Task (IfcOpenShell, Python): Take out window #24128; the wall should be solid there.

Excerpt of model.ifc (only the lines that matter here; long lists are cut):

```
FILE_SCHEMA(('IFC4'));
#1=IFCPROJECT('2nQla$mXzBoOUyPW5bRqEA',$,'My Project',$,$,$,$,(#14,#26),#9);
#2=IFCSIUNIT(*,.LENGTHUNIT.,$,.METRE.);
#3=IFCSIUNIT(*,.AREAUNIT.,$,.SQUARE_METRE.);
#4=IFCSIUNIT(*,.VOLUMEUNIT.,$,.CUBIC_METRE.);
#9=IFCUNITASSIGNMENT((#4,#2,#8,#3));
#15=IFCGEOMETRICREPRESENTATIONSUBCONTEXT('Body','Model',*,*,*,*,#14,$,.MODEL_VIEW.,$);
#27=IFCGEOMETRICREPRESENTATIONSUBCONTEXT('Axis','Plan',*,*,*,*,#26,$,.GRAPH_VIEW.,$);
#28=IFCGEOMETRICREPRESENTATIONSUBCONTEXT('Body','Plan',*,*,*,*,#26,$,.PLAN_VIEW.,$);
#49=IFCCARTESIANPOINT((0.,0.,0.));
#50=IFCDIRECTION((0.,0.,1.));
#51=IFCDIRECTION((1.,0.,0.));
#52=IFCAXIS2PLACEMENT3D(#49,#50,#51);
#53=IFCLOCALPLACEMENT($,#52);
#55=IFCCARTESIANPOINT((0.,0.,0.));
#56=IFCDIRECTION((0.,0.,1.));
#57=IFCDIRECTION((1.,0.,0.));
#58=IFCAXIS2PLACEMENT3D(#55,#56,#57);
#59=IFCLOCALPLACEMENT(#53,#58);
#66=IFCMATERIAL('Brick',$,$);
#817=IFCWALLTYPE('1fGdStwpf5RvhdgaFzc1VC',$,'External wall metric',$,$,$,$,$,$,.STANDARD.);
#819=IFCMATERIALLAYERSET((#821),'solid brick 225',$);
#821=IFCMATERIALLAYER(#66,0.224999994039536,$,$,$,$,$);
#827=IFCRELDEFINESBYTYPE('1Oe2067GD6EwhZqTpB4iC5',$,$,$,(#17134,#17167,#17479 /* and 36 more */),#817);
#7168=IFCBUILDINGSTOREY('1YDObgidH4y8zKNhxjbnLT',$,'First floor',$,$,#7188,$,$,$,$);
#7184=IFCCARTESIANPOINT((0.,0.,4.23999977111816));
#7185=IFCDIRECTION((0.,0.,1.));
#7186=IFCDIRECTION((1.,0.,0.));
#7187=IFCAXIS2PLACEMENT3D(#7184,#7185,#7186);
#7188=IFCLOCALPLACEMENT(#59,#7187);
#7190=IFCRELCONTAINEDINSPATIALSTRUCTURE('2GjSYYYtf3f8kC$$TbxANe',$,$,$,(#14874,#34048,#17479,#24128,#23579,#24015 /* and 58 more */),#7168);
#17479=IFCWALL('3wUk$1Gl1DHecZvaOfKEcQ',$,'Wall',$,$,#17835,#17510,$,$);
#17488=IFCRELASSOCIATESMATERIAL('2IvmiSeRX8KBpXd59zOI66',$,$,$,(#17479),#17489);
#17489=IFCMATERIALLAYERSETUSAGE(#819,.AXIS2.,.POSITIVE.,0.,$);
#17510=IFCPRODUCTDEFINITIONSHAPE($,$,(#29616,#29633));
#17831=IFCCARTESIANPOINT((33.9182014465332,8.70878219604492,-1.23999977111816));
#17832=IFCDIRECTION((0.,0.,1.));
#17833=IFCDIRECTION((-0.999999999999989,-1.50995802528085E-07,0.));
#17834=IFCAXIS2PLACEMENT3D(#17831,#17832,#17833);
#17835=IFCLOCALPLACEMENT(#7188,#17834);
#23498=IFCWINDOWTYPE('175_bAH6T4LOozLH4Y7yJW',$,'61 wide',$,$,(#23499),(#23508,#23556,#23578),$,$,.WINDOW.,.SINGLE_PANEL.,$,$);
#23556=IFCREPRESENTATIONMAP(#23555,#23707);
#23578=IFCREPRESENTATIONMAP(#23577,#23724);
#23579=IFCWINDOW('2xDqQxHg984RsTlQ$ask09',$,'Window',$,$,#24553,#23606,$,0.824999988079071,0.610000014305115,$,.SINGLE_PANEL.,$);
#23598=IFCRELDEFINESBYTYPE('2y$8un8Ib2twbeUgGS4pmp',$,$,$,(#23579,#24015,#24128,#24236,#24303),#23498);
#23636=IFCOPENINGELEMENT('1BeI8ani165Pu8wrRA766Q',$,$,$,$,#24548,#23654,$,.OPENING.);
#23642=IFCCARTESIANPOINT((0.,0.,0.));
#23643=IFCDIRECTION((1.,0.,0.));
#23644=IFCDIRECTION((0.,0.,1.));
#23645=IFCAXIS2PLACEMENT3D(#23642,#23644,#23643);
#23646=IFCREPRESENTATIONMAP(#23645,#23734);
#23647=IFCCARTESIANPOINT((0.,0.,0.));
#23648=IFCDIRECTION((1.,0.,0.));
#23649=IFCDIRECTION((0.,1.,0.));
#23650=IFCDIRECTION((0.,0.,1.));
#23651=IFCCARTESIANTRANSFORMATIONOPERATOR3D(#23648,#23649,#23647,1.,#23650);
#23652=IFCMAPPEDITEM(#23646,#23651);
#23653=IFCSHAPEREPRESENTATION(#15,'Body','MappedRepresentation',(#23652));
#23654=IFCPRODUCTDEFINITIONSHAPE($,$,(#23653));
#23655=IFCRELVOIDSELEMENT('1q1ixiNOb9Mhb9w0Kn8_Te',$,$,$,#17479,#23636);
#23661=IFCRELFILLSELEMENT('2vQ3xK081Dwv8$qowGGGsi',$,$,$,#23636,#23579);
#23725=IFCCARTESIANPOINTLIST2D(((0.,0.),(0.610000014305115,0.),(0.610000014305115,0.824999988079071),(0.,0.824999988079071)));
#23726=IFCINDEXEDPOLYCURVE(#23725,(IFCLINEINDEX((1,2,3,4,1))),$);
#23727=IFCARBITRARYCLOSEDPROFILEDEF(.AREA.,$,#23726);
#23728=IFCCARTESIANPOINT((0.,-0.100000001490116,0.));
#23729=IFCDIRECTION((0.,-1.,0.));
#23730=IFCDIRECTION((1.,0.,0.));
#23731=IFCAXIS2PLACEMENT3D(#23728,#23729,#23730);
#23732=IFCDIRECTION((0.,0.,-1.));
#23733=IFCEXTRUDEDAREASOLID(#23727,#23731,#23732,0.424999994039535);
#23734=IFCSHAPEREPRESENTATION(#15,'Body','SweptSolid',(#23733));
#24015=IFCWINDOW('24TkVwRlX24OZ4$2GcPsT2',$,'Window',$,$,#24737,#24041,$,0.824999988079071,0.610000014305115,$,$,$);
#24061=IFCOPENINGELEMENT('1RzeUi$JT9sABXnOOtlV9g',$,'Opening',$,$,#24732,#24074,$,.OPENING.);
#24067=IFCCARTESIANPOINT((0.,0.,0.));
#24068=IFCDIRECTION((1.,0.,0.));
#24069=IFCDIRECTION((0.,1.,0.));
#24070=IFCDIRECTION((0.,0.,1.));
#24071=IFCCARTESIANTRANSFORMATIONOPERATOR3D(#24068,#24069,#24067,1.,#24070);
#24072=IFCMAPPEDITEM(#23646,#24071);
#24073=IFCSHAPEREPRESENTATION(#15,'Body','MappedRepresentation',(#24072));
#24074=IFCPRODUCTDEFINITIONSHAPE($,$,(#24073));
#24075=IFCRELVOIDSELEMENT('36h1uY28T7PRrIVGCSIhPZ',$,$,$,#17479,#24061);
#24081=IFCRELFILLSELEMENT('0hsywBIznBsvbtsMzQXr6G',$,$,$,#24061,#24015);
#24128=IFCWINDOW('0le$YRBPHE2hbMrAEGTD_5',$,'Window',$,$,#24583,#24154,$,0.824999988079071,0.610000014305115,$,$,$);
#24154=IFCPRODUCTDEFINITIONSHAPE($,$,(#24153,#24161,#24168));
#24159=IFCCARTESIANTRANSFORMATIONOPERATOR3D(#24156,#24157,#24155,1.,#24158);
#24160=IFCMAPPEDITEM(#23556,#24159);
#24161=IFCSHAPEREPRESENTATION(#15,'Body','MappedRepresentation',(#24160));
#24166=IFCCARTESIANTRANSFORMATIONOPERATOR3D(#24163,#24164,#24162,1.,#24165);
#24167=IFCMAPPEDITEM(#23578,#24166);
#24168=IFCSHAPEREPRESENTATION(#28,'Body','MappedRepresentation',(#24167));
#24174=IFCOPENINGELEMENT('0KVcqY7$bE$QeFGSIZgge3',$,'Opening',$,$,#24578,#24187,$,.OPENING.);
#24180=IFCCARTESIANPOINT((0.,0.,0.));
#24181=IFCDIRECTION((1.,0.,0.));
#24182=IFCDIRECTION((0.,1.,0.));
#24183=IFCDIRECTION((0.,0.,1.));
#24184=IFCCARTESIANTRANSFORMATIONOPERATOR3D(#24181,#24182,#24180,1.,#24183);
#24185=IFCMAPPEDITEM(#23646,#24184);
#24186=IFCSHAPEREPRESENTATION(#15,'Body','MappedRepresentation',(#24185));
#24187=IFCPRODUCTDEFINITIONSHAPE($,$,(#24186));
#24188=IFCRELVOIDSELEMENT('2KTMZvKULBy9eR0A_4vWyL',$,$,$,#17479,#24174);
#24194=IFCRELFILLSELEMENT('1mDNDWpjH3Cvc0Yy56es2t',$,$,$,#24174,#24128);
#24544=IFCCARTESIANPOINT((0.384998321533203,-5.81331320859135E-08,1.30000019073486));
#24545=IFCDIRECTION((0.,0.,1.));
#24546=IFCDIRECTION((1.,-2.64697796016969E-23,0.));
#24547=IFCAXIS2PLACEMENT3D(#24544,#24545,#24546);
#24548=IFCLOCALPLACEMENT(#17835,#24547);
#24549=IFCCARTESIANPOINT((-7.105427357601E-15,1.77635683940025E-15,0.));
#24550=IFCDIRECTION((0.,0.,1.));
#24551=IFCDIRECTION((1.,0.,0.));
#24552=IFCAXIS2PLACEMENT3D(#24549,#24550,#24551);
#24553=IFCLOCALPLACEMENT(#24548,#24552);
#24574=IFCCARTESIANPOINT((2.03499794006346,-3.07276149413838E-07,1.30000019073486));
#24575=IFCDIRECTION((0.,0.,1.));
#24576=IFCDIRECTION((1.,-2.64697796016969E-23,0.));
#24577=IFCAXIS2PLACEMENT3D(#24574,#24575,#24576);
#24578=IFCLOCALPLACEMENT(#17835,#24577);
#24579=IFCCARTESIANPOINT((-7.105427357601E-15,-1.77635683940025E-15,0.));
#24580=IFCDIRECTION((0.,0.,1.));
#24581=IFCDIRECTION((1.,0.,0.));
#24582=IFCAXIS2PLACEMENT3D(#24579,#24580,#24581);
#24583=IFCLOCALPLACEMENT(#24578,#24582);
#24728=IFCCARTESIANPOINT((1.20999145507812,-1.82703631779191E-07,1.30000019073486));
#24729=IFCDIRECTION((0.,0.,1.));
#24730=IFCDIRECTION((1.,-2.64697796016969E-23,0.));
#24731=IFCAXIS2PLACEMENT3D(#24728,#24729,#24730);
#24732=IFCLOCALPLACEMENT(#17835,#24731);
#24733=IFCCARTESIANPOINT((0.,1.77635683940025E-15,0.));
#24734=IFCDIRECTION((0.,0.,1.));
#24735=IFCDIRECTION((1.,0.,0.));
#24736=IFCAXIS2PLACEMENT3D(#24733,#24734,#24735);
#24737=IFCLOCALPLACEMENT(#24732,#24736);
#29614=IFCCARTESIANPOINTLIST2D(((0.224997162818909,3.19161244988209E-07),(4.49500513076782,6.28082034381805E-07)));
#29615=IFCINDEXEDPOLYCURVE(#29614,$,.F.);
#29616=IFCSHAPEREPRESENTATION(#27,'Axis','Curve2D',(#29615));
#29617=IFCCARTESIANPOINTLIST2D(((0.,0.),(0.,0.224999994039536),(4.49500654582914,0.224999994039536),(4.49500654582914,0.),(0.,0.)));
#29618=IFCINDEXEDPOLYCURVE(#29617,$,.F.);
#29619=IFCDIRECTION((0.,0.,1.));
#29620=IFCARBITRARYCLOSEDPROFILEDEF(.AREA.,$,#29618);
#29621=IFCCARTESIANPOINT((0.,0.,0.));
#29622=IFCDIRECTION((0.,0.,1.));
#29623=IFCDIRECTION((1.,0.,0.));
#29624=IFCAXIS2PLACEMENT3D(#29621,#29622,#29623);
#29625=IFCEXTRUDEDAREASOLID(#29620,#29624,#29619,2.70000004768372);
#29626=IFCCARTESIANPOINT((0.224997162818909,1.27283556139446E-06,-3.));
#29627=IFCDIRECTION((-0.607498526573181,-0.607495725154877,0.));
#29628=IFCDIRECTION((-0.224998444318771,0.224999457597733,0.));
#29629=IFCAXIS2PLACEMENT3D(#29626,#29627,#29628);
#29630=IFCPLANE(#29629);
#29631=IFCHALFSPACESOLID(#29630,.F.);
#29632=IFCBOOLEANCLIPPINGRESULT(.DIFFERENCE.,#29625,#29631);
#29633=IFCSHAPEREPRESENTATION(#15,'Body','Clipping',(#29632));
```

```python
import ifcopenshell
import ifcopenshell.api.feature
import ifcopenshell.api.root
import ifcopenshell.geom
import ifcopenshell.util.shape

model = ifcopenshell.open("model.ifc")
settings = ifcopenshell.geom.settings()


def volume(element):
    """Net volume in cubic metres, openings subtracted."""
    shape = ifcopenshell.geom.create_shape(settings, element)
    return ifcopenshell.util.shape.get_volume(shape.geometry)


window = model.by_guid("0le$YRBPHE2hbMrAEGTD_5")
opening = window.FillsVoids[0].RelatingOpeningElement
wall = opening.VoidsElements[0].RelatingBuildingElement
before = volume(wall)

ifcopenshell.api.root.remove_product(model, product=window)
ifcopenshell.api.feature.remove_feature(model, feature=opening)

after = volume(wall)

print(f"wall volume {before:.3f} -> {after:.3f} m3")

model.write("model_updated.ifc")
```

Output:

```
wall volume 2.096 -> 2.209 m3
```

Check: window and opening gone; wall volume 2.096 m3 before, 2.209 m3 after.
